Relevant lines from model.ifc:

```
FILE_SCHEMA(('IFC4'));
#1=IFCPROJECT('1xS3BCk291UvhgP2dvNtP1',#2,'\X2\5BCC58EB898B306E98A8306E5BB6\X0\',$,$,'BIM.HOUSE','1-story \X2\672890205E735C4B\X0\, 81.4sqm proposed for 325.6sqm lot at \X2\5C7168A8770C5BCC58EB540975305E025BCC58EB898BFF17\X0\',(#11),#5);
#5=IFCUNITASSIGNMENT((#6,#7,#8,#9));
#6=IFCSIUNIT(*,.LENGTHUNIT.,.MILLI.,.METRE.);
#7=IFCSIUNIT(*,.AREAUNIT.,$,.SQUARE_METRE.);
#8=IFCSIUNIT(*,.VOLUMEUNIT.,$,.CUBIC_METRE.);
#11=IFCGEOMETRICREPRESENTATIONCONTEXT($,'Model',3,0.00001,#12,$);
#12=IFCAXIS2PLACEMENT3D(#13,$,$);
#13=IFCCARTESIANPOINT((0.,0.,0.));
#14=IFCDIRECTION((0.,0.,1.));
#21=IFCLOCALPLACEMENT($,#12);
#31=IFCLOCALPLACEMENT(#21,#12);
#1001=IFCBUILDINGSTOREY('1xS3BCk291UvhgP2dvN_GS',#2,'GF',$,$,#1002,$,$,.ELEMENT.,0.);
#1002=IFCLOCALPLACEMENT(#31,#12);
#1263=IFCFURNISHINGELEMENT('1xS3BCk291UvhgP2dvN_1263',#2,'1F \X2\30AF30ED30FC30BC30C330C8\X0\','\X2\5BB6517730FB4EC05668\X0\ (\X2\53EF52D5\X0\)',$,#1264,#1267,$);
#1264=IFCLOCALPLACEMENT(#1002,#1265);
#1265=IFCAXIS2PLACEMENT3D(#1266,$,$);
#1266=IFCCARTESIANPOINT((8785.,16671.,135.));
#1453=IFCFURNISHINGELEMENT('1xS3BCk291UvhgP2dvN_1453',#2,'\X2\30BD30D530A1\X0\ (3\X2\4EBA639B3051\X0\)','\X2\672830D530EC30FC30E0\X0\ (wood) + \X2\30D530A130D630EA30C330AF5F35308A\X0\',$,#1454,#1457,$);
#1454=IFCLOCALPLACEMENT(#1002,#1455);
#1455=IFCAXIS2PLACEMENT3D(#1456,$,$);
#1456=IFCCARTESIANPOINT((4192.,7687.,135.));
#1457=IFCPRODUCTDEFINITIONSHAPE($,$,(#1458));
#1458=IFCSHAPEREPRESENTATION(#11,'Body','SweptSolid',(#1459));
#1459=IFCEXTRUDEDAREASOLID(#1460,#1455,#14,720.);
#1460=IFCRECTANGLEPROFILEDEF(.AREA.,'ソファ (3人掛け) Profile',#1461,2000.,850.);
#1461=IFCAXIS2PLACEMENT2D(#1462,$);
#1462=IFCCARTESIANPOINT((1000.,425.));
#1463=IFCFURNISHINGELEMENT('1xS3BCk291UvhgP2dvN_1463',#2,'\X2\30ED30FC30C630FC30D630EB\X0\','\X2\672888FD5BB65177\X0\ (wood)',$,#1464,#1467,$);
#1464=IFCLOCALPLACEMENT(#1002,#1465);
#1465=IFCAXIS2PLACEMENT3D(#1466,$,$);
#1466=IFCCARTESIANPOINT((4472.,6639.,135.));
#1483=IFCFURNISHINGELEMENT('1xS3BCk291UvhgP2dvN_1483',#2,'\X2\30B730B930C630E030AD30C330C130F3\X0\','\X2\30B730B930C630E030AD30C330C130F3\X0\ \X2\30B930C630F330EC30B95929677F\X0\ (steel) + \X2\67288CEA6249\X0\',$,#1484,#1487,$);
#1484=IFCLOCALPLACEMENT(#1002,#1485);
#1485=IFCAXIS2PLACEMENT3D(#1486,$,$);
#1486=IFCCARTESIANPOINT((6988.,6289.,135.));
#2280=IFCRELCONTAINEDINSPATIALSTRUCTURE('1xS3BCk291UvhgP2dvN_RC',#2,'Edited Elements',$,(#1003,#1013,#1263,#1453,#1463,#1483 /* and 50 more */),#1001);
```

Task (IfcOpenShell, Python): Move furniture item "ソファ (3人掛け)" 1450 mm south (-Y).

```python
import ifcopenshell
import ifcopenshell.api.geometry
import ifcopenshell.util.placement

model = ifcopenshell.open("model.ifc")

item = model.by_guid("1xS3BCk291UvhgP2dvN_1453")
matrix = ifcopenshell.util.placement.get_local_placement(item.ObjectPlacement)
matrix[1, 3] -= 1450.0
ifcopenshell.api.geometry.edit_object_placement(model, product=item, matrix=matrix, is_si=False)

print(ifcopenshell.util.placement.get_local_placement(item.ObjectPlacement).round(3) + 0.0)

model.write("model-out.ifc")
```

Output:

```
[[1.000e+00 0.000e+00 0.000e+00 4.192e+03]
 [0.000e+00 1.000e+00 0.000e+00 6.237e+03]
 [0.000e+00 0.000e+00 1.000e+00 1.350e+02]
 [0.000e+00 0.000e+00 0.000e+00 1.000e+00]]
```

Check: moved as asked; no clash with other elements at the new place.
